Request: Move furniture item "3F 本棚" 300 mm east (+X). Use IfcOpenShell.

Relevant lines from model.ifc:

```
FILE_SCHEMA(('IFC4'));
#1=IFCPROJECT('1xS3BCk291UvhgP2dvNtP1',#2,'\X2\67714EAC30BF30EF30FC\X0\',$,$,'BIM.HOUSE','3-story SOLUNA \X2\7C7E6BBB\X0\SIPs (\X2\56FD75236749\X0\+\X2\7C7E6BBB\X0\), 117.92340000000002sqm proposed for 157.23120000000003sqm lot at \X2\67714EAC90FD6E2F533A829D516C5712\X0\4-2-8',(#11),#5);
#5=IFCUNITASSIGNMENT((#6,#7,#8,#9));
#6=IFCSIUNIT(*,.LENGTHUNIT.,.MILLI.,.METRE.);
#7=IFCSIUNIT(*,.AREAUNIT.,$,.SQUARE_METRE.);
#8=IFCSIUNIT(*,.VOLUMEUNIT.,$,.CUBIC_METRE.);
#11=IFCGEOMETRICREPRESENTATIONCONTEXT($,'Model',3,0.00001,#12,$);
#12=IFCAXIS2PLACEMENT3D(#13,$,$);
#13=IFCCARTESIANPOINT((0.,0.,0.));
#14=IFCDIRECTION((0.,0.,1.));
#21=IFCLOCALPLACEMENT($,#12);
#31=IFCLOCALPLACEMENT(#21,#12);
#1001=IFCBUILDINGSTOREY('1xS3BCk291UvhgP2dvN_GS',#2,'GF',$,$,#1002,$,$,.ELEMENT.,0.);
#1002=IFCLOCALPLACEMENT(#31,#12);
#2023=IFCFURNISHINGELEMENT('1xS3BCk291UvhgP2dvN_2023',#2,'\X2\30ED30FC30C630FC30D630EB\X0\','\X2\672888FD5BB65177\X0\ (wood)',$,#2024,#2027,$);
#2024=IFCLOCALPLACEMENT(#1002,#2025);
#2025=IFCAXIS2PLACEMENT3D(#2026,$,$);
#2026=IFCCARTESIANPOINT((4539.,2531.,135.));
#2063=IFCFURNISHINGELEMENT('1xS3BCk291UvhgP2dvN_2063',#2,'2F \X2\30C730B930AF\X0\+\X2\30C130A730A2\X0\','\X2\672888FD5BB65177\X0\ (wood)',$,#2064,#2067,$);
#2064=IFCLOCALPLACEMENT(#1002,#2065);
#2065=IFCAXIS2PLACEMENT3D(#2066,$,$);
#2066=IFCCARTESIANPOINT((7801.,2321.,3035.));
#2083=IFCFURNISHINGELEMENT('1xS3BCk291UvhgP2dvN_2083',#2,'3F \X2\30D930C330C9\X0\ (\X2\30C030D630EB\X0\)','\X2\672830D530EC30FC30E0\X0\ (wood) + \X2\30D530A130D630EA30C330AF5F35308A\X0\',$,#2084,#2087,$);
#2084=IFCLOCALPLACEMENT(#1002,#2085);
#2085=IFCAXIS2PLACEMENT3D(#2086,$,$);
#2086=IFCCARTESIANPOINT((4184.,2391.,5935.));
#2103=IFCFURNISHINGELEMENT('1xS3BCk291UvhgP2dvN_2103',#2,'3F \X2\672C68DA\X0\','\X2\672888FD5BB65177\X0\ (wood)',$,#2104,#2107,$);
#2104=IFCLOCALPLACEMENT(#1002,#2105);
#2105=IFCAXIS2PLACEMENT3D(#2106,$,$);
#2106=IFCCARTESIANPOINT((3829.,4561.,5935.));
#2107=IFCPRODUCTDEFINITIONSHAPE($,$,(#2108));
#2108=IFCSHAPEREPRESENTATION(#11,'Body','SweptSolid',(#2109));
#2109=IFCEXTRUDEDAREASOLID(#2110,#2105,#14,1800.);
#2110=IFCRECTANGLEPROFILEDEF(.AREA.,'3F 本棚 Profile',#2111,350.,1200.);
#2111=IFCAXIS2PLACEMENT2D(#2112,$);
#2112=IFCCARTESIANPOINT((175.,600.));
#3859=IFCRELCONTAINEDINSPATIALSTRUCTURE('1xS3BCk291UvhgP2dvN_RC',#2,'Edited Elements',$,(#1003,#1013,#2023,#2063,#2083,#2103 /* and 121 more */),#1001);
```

```python
import ifcopenshell
import ifcopenshell.api.geometry
import ifcopenshell.util.placement
import ifcopenshell.util.unit

model = ifcopenshell.open("model.ifc")
unit_scale = ifcopenshell.util.unit.calculate_unit_scale(model)

item = model.by_guid("1xS3BCk291UvhgP2dvN_2103")
matrix = ifcopenshell.util.placement.get_local_placement(item.ObjectPlacement)
matrix[0, 3] += 0.3 / unit_scale
ifcopenshell.api.geometry.edit_object_placement(model, product=item, matrix=matrix, is_si=False)

print(ifcopenshell.util.placement.get_local_placement(item.ObjectPlacement).round(3) + 0.0)

model.write("model_edited.ifc")
```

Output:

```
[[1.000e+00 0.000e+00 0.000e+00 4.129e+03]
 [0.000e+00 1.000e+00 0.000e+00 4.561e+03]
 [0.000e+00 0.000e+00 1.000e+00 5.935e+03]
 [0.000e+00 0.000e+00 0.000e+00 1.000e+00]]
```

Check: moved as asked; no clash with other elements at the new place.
